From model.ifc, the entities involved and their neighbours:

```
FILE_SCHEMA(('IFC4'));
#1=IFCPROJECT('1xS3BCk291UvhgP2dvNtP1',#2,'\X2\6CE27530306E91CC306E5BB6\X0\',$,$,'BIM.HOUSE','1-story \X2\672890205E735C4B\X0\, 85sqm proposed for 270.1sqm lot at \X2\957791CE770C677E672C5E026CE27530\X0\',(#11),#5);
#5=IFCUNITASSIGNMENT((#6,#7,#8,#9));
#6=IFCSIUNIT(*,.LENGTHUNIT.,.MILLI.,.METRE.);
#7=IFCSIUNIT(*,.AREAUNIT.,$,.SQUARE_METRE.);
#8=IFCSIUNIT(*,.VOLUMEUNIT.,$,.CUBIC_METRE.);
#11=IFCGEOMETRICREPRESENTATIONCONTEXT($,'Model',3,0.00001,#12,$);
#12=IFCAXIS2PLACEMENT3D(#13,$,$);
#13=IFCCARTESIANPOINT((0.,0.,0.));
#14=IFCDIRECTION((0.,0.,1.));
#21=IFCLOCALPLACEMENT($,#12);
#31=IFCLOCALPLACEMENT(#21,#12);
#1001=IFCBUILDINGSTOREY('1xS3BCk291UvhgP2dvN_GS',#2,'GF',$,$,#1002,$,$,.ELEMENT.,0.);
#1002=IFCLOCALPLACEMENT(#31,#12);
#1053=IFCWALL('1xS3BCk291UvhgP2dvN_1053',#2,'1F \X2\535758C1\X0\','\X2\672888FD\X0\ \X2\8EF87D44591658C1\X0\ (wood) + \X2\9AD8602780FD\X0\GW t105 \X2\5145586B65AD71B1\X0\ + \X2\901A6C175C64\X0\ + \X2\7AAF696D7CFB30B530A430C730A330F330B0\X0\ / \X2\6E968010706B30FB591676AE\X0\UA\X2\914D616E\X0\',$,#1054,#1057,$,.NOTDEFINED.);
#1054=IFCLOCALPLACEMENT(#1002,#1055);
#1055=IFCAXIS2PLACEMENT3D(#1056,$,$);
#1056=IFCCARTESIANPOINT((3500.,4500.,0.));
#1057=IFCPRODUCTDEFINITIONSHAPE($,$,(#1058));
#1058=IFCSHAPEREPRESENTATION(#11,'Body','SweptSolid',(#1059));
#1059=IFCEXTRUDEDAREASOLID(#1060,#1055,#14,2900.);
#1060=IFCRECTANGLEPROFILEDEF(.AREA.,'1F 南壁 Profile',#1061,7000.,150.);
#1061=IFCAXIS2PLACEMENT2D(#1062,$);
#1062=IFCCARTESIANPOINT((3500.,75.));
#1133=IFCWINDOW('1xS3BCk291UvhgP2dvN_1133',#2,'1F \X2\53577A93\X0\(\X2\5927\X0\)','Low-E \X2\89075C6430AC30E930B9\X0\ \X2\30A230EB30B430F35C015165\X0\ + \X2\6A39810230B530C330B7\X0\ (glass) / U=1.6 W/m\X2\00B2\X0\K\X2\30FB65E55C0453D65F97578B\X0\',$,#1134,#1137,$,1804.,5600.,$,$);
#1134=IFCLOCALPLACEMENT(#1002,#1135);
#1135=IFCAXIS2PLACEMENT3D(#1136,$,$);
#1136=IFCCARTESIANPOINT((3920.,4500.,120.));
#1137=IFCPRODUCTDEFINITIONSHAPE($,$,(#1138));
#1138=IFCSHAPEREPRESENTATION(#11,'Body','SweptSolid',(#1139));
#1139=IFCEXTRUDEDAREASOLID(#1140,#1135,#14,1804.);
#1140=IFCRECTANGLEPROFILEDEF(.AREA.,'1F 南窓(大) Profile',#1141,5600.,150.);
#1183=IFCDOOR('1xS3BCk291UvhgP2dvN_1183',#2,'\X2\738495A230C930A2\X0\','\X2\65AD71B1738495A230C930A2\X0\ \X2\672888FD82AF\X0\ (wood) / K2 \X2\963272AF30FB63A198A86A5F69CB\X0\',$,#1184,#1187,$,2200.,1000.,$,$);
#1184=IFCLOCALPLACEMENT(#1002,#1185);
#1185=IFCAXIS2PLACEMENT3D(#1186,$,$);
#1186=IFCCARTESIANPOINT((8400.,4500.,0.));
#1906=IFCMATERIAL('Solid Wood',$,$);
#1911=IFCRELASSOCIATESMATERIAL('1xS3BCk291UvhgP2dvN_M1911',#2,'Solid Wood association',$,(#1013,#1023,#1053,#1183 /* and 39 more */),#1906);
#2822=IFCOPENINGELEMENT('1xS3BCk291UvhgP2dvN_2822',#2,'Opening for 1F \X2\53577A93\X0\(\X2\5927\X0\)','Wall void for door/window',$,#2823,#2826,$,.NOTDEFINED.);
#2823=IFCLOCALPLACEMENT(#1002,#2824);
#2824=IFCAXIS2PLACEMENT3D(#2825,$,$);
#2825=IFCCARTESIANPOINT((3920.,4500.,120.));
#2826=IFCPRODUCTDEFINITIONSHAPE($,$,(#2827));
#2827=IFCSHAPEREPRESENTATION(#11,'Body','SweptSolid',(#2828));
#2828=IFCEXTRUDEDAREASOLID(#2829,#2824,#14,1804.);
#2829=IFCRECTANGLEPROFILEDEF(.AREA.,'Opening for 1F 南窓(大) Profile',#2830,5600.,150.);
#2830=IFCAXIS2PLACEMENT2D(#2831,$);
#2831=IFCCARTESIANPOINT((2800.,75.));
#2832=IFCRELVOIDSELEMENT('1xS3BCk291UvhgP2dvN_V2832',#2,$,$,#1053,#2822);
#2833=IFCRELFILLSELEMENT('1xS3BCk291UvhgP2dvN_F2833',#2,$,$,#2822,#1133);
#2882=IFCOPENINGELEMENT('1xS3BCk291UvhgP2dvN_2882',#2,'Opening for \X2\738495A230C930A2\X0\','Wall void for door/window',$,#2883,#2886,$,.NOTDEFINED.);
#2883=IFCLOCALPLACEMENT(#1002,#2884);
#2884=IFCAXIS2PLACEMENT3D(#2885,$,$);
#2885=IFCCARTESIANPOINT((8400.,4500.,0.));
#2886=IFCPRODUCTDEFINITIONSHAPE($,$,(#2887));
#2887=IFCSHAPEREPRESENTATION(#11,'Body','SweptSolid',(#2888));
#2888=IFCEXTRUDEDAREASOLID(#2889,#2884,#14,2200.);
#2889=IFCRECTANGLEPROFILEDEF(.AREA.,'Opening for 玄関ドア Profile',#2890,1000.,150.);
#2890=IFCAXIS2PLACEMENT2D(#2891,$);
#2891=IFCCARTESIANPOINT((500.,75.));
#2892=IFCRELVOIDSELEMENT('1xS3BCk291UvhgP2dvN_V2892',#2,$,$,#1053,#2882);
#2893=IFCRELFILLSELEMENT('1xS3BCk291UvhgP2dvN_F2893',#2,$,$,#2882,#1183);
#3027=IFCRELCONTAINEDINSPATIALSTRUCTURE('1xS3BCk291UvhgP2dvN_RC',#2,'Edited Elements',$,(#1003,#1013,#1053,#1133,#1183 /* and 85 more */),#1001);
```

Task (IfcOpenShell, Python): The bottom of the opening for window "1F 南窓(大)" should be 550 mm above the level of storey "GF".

```python
import numpy as np
import ifcopenshell
import ifcopenshell.api.geometry
import ifcopenshell.geom
import ifcopenshell.util.element
import ifcopenshell.util.placement
import ifcopenshell.util.shape
import ifcopenshell.util.unit

model = ifcopenshell.open("model.ifc")
unit_scale = ifcopenshell.util.unit.calculate_unit_scale(model)

window = model.by_guid("1xS3BCk291UvhgP2dvN_1133")
opening = window.FillsVoids[0].RelatingOpeningElement
storey = ifcopenshell.util.element.get_container(window, ifc_class="IfcBuildingStorey")
level = ifcopenshell.util.placement.get_local_placement(storey.ObjectPlacement)[2, 3]

# The opening's origin need not be at the sill, so measure its lowest point.
shape = ifcopenshell.geom.create_shape(ifcopenshell.geom.settings(), opening)
bottom = ifcopenshell.util.shape.get_shape_bottom_elevation(shape, shape.geometry) / unit_scale
dz = level + 550.0 - bottom

shift = np.array([0.0, 0.0, dz])
# The window is not placed relative to its opening, so move both.
for product in (opening, window):
    matrix = ifcopenshell.util.placement.get_local_placement(product.ObjectPlacement)
    matrix[:3, 3] += shift
    ifcopenshell.api.geometry.edit_object_placement(model, product=product, matrix=matrix, is_si=False)

print(f"moved by {dz * unit_scale:+.3f} m")

model.write("model-out.ifc")
```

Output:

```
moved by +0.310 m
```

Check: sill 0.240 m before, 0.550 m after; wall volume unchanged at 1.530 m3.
